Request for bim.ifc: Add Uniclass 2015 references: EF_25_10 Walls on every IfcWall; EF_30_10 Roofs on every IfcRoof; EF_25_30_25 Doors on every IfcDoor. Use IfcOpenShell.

First a look at what the model holds.

```python
import ifcopenshell

model = ifcopenshell.open("bim.ifc")
print(model.schema)
print("classifications:", [c.Name for c in model.by_type("IfcClassification")])
for ifc_class in ("IfcDoor", "IfcRoof", "IfcStair", "IfcWall", "IfcWindow"):
    print(ifc_class, len(model.by_type(ifc_class)))
```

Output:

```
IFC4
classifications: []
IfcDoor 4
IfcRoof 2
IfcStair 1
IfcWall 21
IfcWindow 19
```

```python
import ifcopenshell
import ifcopenshell.api.classification

model = ifcopenshell.open("bim.ifc")

system = ifcopenshell.api.classification.add_classification(model, classification="Uniclass 2015")

codes = {
    "IfcWall": ("EF_25_10", "Walls"),
    "IfcRoof": ("EF_30_10", "Roofs"),
    "IfcDoor": ("EF_25_30_25", "Doors"),
}
for ifc_class, (code, name) in codes.items():
    products = model.by_type(ifc_class)
    ifcopenshell.api.classification.add_reference(
        model, products=products, classification=system, identification=code, name=name
    )
    print(code, len(products))

model.write("bim_edited.ifc")
```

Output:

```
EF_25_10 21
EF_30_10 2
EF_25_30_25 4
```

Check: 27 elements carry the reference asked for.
